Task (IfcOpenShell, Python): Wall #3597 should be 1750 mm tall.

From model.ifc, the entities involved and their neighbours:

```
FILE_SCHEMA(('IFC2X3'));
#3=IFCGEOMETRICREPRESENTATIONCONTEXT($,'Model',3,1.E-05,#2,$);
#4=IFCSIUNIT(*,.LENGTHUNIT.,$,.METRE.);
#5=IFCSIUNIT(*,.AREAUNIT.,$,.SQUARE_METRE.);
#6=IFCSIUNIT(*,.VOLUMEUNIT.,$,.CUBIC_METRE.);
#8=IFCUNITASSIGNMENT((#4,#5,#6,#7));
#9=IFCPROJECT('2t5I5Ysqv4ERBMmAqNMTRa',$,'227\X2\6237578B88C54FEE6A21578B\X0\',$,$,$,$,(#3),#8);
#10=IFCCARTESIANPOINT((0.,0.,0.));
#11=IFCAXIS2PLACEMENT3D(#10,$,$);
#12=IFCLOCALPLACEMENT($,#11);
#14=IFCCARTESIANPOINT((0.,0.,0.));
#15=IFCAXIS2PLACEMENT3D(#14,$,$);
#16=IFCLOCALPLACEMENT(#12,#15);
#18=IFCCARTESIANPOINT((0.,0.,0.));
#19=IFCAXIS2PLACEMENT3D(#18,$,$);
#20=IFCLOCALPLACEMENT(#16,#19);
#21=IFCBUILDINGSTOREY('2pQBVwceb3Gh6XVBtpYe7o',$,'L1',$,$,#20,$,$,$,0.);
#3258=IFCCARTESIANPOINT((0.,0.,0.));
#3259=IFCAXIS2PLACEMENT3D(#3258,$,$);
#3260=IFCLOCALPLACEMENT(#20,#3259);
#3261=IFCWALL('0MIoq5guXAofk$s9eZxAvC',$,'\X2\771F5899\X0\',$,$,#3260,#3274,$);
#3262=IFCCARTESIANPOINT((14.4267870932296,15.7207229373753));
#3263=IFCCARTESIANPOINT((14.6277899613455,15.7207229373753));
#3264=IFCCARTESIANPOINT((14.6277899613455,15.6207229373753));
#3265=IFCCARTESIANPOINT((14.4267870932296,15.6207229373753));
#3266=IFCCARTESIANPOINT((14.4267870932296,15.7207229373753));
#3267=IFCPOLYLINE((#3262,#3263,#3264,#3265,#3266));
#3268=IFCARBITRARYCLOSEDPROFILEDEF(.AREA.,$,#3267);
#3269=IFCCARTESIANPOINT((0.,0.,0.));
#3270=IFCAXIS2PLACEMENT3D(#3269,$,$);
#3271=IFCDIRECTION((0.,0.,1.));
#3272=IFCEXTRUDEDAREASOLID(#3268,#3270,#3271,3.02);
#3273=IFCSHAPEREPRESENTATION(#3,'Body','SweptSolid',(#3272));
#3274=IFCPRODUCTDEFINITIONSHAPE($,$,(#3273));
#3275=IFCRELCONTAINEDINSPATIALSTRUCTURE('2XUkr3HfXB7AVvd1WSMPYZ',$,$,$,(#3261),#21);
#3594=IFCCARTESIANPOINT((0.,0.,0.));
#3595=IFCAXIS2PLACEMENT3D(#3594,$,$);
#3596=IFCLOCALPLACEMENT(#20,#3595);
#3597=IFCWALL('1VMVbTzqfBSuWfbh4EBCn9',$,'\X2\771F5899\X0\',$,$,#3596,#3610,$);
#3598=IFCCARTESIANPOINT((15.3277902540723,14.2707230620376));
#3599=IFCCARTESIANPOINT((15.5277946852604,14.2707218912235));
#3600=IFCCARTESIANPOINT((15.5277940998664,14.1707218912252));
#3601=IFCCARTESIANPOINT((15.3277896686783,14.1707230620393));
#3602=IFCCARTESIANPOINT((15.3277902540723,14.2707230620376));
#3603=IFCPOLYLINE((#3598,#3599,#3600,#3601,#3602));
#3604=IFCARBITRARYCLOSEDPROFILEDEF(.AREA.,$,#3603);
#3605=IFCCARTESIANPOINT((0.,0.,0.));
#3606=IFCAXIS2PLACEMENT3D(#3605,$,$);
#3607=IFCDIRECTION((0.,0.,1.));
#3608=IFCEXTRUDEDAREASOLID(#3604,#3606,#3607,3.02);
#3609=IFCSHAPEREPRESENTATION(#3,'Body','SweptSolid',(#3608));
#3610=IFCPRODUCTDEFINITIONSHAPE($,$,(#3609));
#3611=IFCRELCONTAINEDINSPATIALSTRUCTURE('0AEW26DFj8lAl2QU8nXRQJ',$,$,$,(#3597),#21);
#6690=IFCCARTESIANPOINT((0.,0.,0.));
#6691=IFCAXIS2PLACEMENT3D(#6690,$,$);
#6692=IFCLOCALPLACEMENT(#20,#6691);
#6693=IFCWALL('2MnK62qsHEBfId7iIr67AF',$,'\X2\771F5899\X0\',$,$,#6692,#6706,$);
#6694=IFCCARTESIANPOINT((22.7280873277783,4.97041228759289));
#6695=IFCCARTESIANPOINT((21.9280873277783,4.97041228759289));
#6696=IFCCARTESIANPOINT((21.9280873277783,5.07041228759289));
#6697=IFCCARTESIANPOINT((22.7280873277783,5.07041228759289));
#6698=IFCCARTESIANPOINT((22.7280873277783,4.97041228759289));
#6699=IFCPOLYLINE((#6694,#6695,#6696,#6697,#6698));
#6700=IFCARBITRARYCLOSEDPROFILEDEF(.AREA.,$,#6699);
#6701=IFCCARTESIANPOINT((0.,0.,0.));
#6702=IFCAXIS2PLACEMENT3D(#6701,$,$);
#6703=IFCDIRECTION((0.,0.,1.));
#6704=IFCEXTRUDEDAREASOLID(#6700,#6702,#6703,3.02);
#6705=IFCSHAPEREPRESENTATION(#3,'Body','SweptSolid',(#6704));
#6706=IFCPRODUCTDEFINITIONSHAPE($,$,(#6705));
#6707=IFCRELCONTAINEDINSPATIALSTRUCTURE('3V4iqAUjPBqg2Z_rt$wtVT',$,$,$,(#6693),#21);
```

```python
import ifcopenshell
import ifcopenshell.geom
import ifcopenshell.util.shape
import ifcopenshell.util.unit

model = ifcopenshell.open("model.ifc")
unit_scale = ifcopenshell.util.unit.calculate_unit_scale(model)
settings = ifcopenshell.geom.settings()


def volume(element):
    """Net volume in cubic metres, openings subtracted."""
    shape = ifcopenshell.geom.create_shape(settings, element)
    return ifcopenshell.util.shape.get_volume(shape.geometry)


wall = model.by_guid("1VMVbTzqfBSuWfbh4EBCn9")
before = volume(wall)

body = next(r for r in wall.Representation.Representations if r.RepresentationIdentifier == "Body")
solid = body.Items[0]
old_height = solid.Depth
solid.Depth = 1.75 / unit_scale
after = volume(wall)

print(f"height {old_height:g} -> {solid.Depth:g}, volume {before:.3f} -> {after:.3f} m3")

model.write("model_v2.ifc")
```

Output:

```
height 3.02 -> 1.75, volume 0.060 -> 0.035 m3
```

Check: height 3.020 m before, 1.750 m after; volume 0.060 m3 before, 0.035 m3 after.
